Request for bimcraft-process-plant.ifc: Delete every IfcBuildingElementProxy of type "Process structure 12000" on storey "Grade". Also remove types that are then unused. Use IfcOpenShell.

First a look at what the model holds.

```python
import ifcopenshell
import ifcopenshell.util.element

model = ifcopenshell.open("bimcraft-process-plant.ifc")
print(model.schema)
storey = next(s for s in model.by_type("IfcBuildingStorey") if s.Name == "Grade")
proxies = [e for e in ifcopenshell.util.element.get_decomposition(storey) if e.is_a("IfcBuildingElementProxy")]
seen = {}
for e in proxies:
    element_type = ifcopenshell.util.element.get_type(e)
    name = element_type.Name if element_type not in (None, e) else None
    seen[name] = seen.get(name, 0) + 1
for name, count in sorted(seen.items(), key=str):
    print(count, "x", name)
```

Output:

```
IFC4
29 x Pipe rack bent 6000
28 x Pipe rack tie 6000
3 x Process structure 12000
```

```python
import ifcopenshell
import ifcopenshell.api.root
import ifcopenshell.util.element

model = ifcopenshell.open("bimcraft-process-plant.ifc")

storey = next(s for s in model.by_type("IfcBuildingStorey") if s.Name == "Grade")
proxies = [e for e in ifcopenshell.util.element.get_decomposition(storey) if e.is_a("IfcBuildingElementProxy")]
targets = [e for e in proxies if (t := ifcopenshell.util.element.get_type(e)) not in (None, e) and t.Name == "Process structure 12000"]
types = {ifcopenshell.util.element.get_type(e) for e in targets} - {None, *targets}

for e in targets:
    ifcopenshell.api.root.remove_product(model, product=e)
print(len(targets), "removed")

unused = [t for t in types if not ifcopenshell.util.element.get_types(t)]
for t in unused:
    ifcopenshell.api.root.remove_product(model, product=t)
print(len(unused), "unused types removed")

model.write("bimcraft-process-plant-out.ifc")
```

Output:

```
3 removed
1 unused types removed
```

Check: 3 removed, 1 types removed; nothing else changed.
